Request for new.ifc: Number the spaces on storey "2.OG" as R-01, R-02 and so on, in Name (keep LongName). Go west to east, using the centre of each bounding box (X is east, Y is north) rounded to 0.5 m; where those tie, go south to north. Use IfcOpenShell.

First a look at what the model holds.

```python
import ifcopenshell
import ifcopenshell.util.element
import ifcopenshell.util.placement

model = ifcopenshell.open("new.ifc")
print(model.schema)
storey = next(s for s in model.by_type("IfcBuildingStorey") if s.Name == "2.OG")
spaces = [e for e in ifcopenshell.util.element.get_decomposition(storey) if e.is_a("IfcSpace")]
for e in sorted(spaces, key=lambda e: e.id()):
    origin = ifcopenshell.util.placement.get_local_placement(e.ObjectPlacement)[:3, 3]
    print(e.id(), e.Name, e.LongName, origin.round(2) + 0.0, sep=" | ")
```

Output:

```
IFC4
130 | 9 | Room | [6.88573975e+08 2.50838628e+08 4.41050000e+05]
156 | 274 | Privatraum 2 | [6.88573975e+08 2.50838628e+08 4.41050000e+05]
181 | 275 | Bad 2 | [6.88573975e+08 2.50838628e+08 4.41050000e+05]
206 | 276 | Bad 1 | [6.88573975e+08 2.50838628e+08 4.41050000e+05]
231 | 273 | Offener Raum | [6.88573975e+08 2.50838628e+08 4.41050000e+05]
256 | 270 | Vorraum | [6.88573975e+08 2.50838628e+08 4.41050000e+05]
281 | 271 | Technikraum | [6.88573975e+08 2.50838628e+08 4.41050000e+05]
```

```python
import ifcopenshell
import ifcopenshell.geom
import ifcopenshell.util.element
import ifcopenshell.util.shape

model = ifcopenshell.open("new.ifc")
settings = ifcopenshell.geom.settings()
settings.set("use-world-coords", True)


def centre(element):
    shape = ifcopenshell.geom.create_shape(settings, element)
    return ifcopenshell.util.shape.get_bbox_centroid(shape.geometry)


storey = next(s for s in model.by_type("IfcBuildingStorey") if s.Name == "2.OG")
spaces = [e for e in ifcopenshell.util.element.get_decomposition(storey) if e.is_a("IfcSpace")]

# Insertion points can sit at a corner or the storey origin, so sort by the geometry (in metres).
centres = {e: centre(e) for e in spaces}
spaces.sort(key=lambda e: (round(centres[e][0] / 0.5), centres[e][1]))

for i, e in enumerate(spaces, start=1):
    number = f"R-{i:02d}"
    e.Name = number
    print(e.id(), number)

model.write("new-out.ifc")
```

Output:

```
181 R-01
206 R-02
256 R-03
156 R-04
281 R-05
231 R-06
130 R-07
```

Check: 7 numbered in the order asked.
